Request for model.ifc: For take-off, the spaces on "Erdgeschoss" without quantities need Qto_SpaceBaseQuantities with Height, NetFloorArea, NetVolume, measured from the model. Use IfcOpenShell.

First a look at what the model holds.

```python
import ifcopenshell
import ifcopenshell.util.element
import ifcopenshell.util.unit

model = ifcopenshell.open("model.ifc")
print(model.schema)
for unit_type in ("LENGTHUNIT", "AREAUNIT", "VOLUMEUNIT"):
    print(unit_type, ifcopenshell.util.unit.calculate_unit_scale(model, unit_type))
storey = next(s for s in model.by_type("IfcBuildingStorey") if s.Name == "Erdgeschoss")
spaces = [e for e in ifcopenshell.util.element.get_decomposition(storey) if e.is_a("IfcSpace")]
for e in sorted(spaces, key=lambda e: e.id()):
    print(e.id(), e.is_a(), e.Name, list(ifcopenshell.util.element.get_psets(e, qtos_only=True)), sep=" | ")
```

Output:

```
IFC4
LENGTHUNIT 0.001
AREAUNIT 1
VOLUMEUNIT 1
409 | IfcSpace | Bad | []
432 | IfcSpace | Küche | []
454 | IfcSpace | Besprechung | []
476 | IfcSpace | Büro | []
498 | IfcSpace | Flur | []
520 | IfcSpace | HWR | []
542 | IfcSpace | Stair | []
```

```python
import ifcopenshell
import ifcopenshell.api.pset
import ifcopenshell.geom
import ifcopenshell.util.element
import ifcopenshell.util.shape
import ifcopenshell.util.unit

model = ifcopenshell.open("model.ifc")
unit_scale = ifcopenshell.util.unit.calculate_unit_scale(model)
area_scale = ifcopenshell.util.unit.calculate_unit_scale(model, "AREAUNIT")
volume_scale = ifcopenshell.util.unit.calculate_unit_scale(model, "VOLUMEUNIT")
settings = ifcopenshell.geom.settings()

storey = next(s for s in model.by_type("IfcBuildingStorey") if s.Name == "Erdgeschoss")
spaces = [e for e in ifcopenshell.util.element.get_decomposition(storey) if e.is_a("IfcSpace")]

for e in sorted(spaces, key=lambda e: e.id()):
    if ifcopenshell.util.element.get_psets(e, qtos_only=True, should_inherit=False):
        continue
    # Geometry comes back in metres, in the element's own axes.
    shape = ifcopenshell.geom.create_shape(settings, e)
    values = {
        "Height": ifcopenshell.util.shape.get_z(shape.geometry) / unit_scale,
        "NetFloorArea": ifcopenshell.util.shape.get_footprint_area(shape.geometry) / area_scale,
        "NetVolume": ifcopenshell.util.shape.get_volume(shape.geometry) / volume_scale,
    }
    qto = ifcopenshell.api.pset.add_qto(model, product=e, name="Qto_SpaceBaseQuantities")
    ifcopenshell.api.pset.edit_qto(model, qto=qto, properties=values)
    print(e.id(), {k: round(v, 3) for k, v in values.items()})

model.write("model_v2.ifc")
```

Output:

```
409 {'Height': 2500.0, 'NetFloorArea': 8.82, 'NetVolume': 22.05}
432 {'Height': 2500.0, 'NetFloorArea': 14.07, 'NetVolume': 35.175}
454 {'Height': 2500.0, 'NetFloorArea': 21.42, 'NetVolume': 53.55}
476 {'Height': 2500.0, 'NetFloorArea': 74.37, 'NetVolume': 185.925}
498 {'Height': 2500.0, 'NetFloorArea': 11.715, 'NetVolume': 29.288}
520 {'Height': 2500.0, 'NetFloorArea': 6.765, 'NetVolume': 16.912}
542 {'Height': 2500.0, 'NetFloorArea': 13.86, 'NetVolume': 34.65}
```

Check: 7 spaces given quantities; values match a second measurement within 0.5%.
